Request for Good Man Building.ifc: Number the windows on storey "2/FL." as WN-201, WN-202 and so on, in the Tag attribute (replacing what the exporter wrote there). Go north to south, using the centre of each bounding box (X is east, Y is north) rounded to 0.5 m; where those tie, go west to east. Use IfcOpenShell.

First a look at what the model holds.

```python
import ifcopenshell
import ifcopenshell.util.element
import ifcopenshell.util.placement

model = ifcopenshell.open("Good Man Building.ifc")
print(model.schema)
storey = next(s for s in model.by_type("IfcBuildingStorey") if s.Name == "2/FL.")
windows = [e for e in ifcopenshell.util.element.get_decomposition(storey) if e.is_a("IfcWindow")]
for e in sorted(windows, key=lambda e: e.id()):
    origin = ifcopenshell.util.placement.get_local_placement(e.ObjectPlacement)[:3, 3]
    print(e.id(), e.Tag, e.Name, origin.round(2) + 0.0, sep=" | ")
```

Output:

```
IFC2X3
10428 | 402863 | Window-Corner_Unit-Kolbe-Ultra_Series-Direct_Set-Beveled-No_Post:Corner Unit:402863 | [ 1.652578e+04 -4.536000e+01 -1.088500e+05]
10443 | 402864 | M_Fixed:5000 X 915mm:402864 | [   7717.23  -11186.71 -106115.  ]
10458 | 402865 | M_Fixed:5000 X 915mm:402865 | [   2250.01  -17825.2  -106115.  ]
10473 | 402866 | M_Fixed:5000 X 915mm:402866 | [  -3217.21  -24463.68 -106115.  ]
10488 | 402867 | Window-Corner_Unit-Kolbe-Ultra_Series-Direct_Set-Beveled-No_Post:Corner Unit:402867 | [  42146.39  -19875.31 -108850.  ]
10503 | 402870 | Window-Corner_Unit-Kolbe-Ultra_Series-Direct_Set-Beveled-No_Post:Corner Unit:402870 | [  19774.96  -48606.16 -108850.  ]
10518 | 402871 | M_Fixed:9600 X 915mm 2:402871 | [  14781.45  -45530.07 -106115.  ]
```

```python
import ifcopenshell
import ifcopenshell.geom
import ifcopenshell.util.element
import ifcopenshell.util.shape

model = ifcopenshell.open("Good Man Building.ifc")
settings = ifcopenshell.geom.settings()
settings.set("use-world-coords", True)


def centre(element):
    shape = ifcopenshell.geom.create_shape(settings, element)
    return ifcopenshell.util.shape.get_bbox_centroid(shape.geometry)


storey = next(s for s in model.by_type("IfcBuildingStorey") if s.Name == "2/FL.")
windows = [e for e in ifcopenshell.util.element.get_decomposition(storey) if e.is_a("IfcWindow")]

# Insertion points can sit at a corner or the storey origin, so sort by the geometry (in metres).
centres = {e: centre(e) for e in windows}
windows.sort(key=lambda e: (-round(centres[e][1] / 0.5), centres[e][0]))

for i, e in enumerate(windows, start=1):
    number = f"WN-2{i:02d}"
    e.Tag = number
    print(e.id(), number)

model.write("Good Man Building_rev.ifc")
```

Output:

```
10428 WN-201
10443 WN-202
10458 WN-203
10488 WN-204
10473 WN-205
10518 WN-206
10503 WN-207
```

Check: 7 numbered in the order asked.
